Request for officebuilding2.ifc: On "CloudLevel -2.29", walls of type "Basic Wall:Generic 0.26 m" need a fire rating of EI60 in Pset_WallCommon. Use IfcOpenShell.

First a look at what the model holds.

```python
import ifcopenshell
import ifcopenshell.util.element

model = ifcopenshell.open("officebuilding2.ifc")
print(model.schema)
storey = next(s for s in model.by_type("IfcBuildingStorey") if s.Name == "CloudLevel -2.29")
walls = [e for e in ifcopenshell.util.element.get_decomposition(storey) if e.is_a("IfcWall")]
seen = {}
for e in walls:
    element_type = ifcopenshell.util.element.get_type(e)
    key = (element_type.Name if element_type != e and element_type else None, ifcopenshell.util.element.get_pset(e, "Pset_WallCommon", "FireRating"))
    seen[key] = seen.get(key, 0) + 1
for (name, value), count in sorted(seen.items(), key=str):
    print(count, "x", name, "|", value)
```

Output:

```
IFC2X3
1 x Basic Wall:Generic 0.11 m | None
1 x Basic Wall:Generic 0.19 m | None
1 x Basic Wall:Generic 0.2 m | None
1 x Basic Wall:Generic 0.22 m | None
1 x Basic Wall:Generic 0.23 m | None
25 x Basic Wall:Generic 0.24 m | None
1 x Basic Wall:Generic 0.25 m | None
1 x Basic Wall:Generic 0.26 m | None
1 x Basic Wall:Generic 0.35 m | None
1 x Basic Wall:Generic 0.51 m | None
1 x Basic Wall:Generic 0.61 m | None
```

```python
import ifcopenshell
import ifcopenshell.api.pset
import ifcopenshell.util.element

model = ifcopenshell.open("officebuilding2.ifc")

storey = next(s for s in model.by_type("IfcBuildingStorey") if s.Name == "CloudLevel -2.29")
walls = [e for e in ifcopenshell.util.element.get_decomposition(storey) if e.is_a("IfcWall")]

count = 0
for e in walls:
    element_type = ifcopenshell.util.element.get_type(e)
    if element_type in (None, e) or element_type.Name != "Basic Wall:Generic 0.26 m":
        continue
    # add_pset returns the element's existing set when there is one.
    pset = ifcopenshell.api.pset.add_pset(model, product=e, name="Pset_WallCommon")
    ifcopenshell.api.pset.edit_pset(model, pset=pset, properties={"FireRating": "EI60"})
    count += 1

print(count, "walls updated")

model.write("officebuilding2-out.ifc")
```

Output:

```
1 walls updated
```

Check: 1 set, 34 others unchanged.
